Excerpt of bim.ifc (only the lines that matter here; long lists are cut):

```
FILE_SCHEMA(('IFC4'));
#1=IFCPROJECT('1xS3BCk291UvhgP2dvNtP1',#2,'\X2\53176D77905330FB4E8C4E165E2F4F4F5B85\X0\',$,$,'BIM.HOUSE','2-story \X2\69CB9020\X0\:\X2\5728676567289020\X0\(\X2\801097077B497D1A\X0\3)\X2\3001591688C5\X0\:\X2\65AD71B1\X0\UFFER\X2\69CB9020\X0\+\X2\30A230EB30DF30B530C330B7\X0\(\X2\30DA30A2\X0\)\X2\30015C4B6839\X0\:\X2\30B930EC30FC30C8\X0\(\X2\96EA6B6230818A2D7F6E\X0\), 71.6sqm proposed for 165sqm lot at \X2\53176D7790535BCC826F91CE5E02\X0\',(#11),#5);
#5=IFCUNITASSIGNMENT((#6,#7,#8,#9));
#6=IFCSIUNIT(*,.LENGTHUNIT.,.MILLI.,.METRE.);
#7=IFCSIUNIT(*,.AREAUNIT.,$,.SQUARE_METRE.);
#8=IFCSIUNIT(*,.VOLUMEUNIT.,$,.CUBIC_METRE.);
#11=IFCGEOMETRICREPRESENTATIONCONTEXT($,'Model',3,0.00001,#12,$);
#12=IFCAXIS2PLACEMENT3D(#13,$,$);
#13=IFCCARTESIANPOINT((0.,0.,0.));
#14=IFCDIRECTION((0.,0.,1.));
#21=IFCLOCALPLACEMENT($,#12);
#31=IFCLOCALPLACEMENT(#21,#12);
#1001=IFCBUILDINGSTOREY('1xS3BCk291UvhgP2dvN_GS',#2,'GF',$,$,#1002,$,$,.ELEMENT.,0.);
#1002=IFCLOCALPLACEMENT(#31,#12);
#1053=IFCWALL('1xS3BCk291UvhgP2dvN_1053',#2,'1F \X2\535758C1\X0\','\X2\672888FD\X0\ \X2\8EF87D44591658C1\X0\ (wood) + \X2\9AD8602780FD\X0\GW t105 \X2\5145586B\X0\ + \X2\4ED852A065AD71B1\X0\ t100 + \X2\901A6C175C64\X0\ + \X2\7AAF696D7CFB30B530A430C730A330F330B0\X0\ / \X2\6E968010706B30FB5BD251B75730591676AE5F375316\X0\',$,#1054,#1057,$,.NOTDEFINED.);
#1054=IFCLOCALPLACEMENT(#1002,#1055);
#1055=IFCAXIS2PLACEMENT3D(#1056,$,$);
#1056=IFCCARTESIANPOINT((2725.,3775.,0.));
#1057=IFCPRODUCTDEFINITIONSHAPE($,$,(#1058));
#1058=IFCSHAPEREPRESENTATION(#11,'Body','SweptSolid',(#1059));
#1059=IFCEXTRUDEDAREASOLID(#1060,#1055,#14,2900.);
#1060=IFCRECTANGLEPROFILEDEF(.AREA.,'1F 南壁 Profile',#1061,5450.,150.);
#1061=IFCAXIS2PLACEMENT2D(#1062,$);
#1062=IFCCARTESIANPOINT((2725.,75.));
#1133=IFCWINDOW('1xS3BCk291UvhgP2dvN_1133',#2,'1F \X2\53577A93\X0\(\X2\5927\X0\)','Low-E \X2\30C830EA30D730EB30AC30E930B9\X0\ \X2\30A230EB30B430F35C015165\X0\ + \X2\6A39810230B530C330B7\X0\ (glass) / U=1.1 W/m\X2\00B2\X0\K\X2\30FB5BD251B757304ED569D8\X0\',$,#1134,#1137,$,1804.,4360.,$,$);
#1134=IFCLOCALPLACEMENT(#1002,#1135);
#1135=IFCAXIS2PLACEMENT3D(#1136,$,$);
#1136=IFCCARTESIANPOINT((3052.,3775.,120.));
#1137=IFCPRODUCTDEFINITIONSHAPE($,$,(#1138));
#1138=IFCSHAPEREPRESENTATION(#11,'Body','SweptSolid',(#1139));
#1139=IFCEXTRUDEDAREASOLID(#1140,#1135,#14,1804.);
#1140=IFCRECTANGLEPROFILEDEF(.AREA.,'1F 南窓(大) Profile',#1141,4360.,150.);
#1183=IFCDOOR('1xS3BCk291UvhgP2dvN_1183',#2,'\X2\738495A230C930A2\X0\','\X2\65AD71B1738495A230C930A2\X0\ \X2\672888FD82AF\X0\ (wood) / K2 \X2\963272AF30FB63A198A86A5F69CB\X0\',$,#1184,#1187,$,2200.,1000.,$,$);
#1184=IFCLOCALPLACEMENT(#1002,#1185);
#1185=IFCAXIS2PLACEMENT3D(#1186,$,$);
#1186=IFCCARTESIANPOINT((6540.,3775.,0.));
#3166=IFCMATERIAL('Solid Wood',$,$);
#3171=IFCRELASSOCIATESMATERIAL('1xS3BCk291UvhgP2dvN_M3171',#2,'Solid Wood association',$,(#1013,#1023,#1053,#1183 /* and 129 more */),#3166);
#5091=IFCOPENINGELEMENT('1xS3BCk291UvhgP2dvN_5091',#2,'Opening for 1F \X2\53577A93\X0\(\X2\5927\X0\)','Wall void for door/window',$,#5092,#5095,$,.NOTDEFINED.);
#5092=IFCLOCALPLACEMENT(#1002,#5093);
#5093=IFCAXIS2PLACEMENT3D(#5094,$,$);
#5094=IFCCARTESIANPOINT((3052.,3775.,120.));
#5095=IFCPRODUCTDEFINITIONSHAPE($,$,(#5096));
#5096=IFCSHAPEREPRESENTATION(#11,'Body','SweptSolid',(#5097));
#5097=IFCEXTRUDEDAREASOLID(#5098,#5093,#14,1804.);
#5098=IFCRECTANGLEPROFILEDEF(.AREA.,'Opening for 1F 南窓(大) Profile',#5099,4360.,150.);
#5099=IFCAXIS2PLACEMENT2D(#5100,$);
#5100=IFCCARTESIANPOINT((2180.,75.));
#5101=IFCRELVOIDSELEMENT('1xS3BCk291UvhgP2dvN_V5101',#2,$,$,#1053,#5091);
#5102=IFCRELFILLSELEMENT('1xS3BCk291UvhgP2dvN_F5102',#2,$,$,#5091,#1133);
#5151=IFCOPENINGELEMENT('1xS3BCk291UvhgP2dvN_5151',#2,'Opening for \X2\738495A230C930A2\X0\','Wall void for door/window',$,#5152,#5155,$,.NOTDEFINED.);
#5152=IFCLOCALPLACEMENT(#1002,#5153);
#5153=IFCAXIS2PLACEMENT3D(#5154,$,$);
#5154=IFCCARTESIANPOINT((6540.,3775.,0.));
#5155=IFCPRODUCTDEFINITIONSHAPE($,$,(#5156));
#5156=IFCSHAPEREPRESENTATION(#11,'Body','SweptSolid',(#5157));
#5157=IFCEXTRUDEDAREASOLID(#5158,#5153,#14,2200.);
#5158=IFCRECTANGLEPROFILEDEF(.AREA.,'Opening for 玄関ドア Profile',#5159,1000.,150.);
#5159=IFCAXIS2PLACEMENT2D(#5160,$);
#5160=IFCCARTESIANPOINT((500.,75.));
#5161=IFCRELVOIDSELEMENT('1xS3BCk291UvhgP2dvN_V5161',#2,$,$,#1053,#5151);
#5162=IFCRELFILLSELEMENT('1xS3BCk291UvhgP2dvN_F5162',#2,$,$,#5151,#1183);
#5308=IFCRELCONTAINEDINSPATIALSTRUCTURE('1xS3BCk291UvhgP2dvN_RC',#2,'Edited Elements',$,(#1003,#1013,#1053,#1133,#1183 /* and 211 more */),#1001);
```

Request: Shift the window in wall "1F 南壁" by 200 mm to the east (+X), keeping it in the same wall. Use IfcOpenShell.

```python
import ifcopenshell
import ifcopenshell.api.geometry
import ifcopenshell.util.placement

model = ifcopenshell.open("bim.ifc")

window = model.by_guid("1xS3BCk291UvhgP2dvN_1133")
opening = window.FillsVoids[0].RelatingOpeningElement
wall = opening.VoidsElements[0].RelatingBuildingElement

wall_matrix = ifcopenshell.util.placement.get_local_placement(wall.ObjectPlacement)
shift = wall_matrix[:3, 0] * 200.0
before = ifcopenshell.util.placement.get_local_placement(window.ObjectPlacement)[:3, 3].copy()

# The window is not placed relative to its opening, so move both.
for product in (opening, window):
    matrix = ifcopenshell.util.placement.get_local_placement(product.ObjectPlacement)
    matrix[:3, 3] += shift
    ifcopenshell.api.geometry.edit_object_placement(model, product=product, matrix=matrix, is_si=False)

after = ifcopenshell.util.placement.get_local_placement(window.ObjectPlacement)[:3, 3]
print("window moved by", (after - before).round(3) + 0.0)

model.write("bim_rev.ifc")
```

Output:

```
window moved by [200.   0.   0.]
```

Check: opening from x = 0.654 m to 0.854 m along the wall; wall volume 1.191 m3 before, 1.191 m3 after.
